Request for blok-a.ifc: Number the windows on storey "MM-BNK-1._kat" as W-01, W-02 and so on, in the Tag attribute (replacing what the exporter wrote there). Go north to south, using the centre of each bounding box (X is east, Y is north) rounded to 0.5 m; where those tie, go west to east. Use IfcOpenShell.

First a look at what the model holds.

```python
import ifcopenshell
import ifcopenshell.util.element
import ifcopenshell.util.placement

model = ifcopenshell.open("blok-a.ifc")
print(model.schema)
storey = next(s for s in model.by_type("IfcBuildingStorey") if s.Name == "MM-BNK-1._kat")
windows = [e for e in ifcopenshell.util.element.get_decomposition(storey) if e.is_a("IfcWindow")]
for e in sorted(windows, key=lambda e: e.id()):
    origin = ifcopenshell.util.placement.get_local_placement(e.ObjectPlacement)[:3, 3]
    print(e.id(), e.Tag, e.Name, origin.round(2) + 0.0, sep=" | ")
```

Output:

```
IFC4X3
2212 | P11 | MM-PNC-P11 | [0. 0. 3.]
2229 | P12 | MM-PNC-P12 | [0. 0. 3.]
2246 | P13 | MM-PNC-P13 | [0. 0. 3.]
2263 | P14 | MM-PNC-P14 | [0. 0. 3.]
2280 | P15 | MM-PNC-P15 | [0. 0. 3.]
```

```python
import ifcopenshell
import ifcopenshell.geom
import ifcopenshell.util.element
import ifcopenshell.util.shape

model = ifcopenshell.open("blok-a.ifc")
settings = ifcopenshell.geom.settings()
settings.set("use-world-coords", True)


def centre(element):
    shape = ifcopenshell.geom.create_shape(settings, element)
    return ifcopenshell.util.shape.get_bbox_centroid(shape.geometry)


storey = next(s for s in model.by_type("IfcBuildingStorey") if s.Name == "MM-BNK-1._kat")
windows = [e for e in ifcopenshell.util.element.get_decomposition(storey) if e.is_a("IfcWindow")]

# Insertion points can sit at a corner or the storey origin, so sort by the geometry (in metres).
centres = {e: centre(e) for e in windows}
windows.sort(key=lambda e: (-round(centres[e][1] / 0.5), centres[e][0]))

for i, e in enumerate(windows, start=1):
    number = f"W-{i:02d}"
    e.Tag = number
    print(e.id(), number)

model.write("blok-a_updated.ifc")
```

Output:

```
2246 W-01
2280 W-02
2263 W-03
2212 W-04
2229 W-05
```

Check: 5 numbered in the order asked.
